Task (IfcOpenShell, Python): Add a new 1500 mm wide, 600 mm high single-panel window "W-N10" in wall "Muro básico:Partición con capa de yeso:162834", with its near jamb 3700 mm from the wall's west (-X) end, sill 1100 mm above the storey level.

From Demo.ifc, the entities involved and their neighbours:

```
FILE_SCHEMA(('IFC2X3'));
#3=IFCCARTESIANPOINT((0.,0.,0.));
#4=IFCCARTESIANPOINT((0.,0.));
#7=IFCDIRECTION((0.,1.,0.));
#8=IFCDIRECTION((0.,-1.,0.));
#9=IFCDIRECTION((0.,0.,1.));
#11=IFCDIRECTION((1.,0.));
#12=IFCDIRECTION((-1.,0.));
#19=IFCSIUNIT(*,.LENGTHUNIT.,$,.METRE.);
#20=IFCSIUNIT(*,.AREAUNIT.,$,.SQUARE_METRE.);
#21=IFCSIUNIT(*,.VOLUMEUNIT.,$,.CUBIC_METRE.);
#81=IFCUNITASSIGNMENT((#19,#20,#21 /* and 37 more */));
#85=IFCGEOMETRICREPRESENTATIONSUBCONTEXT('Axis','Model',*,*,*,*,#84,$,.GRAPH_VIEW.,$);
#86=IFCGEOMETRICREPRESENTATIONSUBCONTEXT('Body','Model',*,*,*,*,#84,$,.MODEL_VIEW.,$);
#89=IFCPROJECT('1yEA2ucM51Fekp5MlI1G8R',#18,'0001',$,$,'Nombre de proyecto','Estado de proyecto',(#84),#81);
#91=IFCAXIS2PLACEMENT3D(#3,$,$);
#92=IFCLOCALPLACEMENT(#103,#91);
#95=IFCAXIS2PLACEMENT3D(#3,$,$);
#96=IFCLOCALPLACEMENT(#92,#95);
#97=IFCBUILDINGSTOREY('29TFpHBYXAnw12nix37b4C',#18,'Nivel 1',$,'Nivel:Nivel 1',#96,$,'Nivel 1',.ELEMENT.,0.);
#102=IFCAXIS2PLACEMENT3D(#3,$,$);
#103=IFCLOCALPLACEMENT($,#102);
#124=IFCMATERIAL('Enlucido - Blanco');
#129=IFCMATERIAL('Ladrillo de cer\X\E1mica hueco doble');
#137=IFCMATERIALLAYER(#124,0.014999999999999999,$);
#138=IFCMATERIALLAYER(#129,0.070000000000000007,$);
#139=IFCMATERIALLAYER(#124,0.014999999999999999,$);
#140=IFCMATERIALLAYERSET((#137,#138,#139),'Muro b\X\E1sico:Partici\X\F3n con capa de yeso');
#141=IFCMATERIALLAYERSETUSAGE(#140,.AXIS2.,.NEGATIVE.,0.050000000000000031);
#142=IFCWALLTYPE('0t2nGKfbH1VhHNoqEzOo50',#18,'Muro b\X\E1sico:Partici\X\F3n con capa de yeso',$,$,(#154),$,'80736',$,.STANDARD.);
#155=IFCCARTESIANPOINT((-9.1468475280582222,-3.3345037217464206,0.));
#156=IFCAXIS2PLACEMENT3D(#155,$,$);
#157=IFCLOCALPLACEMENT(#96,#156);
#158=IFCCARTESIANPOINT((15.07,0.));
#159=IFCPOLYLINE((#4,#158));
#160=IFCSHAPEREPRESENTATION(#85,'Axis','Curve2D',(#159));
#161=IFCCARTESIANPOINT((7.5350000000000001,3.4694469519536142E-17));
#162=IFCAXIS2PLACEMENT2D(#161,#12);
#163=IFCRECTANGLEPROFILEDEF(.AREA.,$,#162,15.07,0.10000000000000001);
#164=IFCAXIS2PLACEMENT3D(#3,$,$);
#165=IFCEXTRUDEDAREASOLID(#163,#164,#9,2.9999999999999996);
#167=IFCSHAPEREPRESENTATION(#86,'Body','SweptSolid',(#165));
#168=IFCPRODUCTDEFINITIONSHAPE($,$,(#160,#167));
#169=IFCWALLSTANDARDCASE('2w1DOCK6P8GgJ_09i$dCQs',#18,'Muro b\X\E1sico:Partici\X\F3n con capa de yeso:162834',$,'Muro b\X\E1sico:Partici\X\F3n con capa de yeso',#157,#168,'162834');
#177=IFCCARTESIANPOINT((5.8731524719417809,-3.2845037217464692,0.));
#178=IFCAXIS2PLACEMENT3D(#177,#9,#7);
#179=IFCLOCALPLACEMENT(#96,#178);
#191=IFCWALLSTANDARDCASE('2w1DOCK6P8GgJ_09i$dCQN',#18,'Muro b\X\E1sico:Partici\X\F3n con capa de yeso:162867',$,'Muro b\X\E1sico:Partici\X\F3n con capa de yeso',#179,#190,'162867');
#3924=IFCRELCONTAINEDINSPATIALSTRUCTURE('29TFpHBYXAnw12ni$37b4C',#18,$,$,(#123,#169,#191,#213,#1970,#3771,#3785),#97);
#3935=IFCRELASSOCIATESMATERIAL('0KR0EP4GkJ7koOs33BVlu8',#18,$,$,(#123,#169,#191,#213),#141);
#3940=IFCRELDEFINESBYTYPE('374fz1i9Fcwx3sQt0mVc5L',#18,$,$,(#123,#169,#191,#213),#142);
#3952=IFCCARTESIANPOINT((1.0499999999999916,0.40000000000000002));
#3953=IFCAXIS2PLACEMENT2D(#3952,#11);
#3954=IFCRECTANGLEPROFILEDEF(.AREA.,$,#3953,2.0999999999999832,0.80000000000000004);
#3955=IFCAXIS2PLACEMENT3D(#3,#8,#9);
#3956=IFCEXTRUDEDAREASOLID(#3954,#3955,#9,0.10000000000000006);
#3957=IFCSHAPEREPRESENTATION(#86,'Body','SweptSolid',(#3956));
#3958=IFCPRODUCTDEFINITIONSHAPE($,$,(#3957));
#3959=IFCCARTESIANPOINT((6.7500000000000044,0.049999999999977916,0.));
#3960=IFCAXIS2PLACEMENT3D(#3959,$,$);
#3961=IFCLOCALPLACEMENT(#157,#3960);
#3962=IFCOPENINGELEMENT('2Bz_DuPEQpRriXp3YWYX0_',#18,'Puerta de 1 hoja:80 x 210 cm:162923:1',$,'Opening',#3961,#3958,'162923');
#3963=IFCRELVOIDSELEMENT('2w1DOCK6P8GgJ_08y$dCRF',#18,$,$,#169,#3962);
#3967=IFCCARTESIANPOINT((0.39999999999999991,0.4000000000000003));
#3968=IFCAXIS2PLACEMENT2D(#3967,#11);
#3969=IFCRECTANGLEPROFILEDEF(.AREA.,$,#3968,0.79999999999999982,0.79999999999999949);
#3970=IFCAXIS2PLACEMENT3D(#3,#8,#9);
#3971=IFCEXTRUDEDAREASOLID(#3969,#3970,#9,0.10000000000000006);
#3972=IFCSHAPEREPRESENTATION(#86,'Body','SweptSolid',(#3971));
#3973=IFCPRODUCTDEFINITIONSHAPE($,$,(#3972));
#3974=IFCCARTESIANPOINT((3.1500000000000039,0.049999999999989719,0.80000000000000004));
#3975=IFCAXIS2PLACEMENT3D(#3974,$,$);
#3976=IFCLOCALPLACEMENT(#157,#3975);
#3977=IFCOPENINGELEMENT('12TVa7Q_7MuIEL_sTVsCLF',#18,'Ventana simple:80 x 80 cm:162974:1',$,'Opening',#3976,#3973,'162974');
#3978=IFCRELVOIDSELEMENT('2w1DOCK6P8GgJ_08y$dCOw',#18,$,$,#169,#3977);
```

```python
import numpy as np
import ifcopenshell
import ifcopenshell.api.feature
import ifcopenshell.api.geometry
import ifcopenshell.api.root
import ifcopenshell.api.spatial
import ifcopenshell.api.type
import ifcopenshell.geom
import ifcopenshell.util.element
import ifcopenshell.util.placement
import ifcopenshell.util.representation
import ifcopenshell.util.shape
import ifcopenshell.util.unit

model = ifcopenshell.open("Demo.ifc")
unit_scale = ifcopenshell.util.unit.calculate_unit_scale(model)
settings = ifcopenshell.geom.settings()


def volume(element):
    """Net volume in cubic metres, openings subtracted."""
    shape = ifcopenshell.geom.create_shape(settings, element)
    return ifcopenshell.util.shape.get_volume(shape.geometry)


wall = model.by_guid("2w1DOCK6P8GgJ_09i$dCQs")
storey = ifcopenshell.util.element.get_container(wall, ifc_class="IfcBuildingStorey")
context = ifcopenshell.util.representation.get_context(model, "Model", "Body", "MODEL_VIEW")
before = volume(wall)

width, height, from_end, sill = 1.5, 0.6, 3.7, 1.1  # metres

# The wall runs along its own X axis, and the end named is its -X end.
wall_shape = ifcopenshell.geom.create_shape(settings, wall)
x, y, z = ifcopenshell.util.shape.get_vertices(wall_shape.geometry).T
start = x.min() + from_end
face, thickness = float(y.min()), float(y.max() - y.min())
wall_matrix = ifcopenshell.util.placement.get_local_placement(wall.ObjectPlacement)
level = ifcopenshell.util.placement.get_local_placement(storey.ObjectPlacement)[2, 3]


def in_wall(x, y):
    """Placement at x, y metres in the wall's axes, at sill height."""
    matrix = wall_matrix.copy()
    matrix[:, 3] = wall_matrix @ np.array([x / unit_scale, y / unit_scale, 0.0, 1.0])
    matrix[2, 3] = level + sill / unit_scale
    return matrix


# Opening: a box that overshoots both wall faces by 50 mm.
opening = ifcopenshell.api.root.create_entity(model, ifc_class="IfcOpeningElement")
box = ifcopenshell.api.geometry.add_wall_representation(
    model, context=context, length=width, height=height, thickness=thickness + 0.1
)
ifcopenshell.api.geometry.assign_representation(model, product=opening, representation=box)
ifcopenshell.api.geometry.edit_object_placement(model, product=opening, matrix=in_wall(start, face - 0.05), is_si=False)
ifcopenshell.api.feature.add_feature(model, feature=opening, element=wall)

window = ifcopenshell.api.root.create_entity(model, ifc_class="IfcWindow", name="W-N10")
window.OverallWidth, window.OverallHeight = width / unit_scale, height / unit_scale
body = ifcopenshell.api.geometry.add_window_representation(
    model,
    context=context,
    overall_width=window.OverallWidth,
    overall_height=window.OverallHeight,
    partition_type="SINGLE_PANEL",
)
ifcopenshell.api.geometry.assign_representation(model, product=window, representation=body)
ifcopenshell.api.spatial.assign_container(model, products=[window], relating_structure=storey)
fills = ifcopenshell.api.feature.add_filling(model, opening=opening, element=window)
fills.OwnerHistory = window.OwnerHistory  # required in IFC2X3

# IFC2X3 keeps the operation on the window style.
style = ifcopenshell.api.root.create_entity(model, ifc_class="IfcWindowStyle", name="W-N10")
style.OperationType, style.ConstructionType = "SINGLE_PANEL", "NOTDEFINED"
style.ParameterTakesPrecedence = style.Sizeable = False
ifcopenshell.api.type.assign_type(model, related_objects=[window], relating_type=style)

# Centre the window in the wall's thickness.
ifcopenshell.api.geometry.edit_object_placement(model, product=window, matrix=in_wall(start, face), is_si=False)
window_shape = ifcopenshell.geom.create_shape(settings, window)
depth = ifcopenshell.util.shape.get_vertices(window_shape.geometry)[:, 1]
offset = face + thickness / 2 - (depth.min() + depth.max()) / 2
ifcopenshell.api.geometry.edit_object_placement(model, product=window, matrix=in_wall(start, offset), is_si=False)

after = volume(wall)

print(f"wall volume {before:.3f} -> {after:.3f} m3")

model.write("Demo_rev.ifc")
```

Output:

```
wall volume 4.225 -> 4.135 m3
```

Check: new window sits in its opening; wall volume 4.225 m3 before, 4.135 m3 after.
